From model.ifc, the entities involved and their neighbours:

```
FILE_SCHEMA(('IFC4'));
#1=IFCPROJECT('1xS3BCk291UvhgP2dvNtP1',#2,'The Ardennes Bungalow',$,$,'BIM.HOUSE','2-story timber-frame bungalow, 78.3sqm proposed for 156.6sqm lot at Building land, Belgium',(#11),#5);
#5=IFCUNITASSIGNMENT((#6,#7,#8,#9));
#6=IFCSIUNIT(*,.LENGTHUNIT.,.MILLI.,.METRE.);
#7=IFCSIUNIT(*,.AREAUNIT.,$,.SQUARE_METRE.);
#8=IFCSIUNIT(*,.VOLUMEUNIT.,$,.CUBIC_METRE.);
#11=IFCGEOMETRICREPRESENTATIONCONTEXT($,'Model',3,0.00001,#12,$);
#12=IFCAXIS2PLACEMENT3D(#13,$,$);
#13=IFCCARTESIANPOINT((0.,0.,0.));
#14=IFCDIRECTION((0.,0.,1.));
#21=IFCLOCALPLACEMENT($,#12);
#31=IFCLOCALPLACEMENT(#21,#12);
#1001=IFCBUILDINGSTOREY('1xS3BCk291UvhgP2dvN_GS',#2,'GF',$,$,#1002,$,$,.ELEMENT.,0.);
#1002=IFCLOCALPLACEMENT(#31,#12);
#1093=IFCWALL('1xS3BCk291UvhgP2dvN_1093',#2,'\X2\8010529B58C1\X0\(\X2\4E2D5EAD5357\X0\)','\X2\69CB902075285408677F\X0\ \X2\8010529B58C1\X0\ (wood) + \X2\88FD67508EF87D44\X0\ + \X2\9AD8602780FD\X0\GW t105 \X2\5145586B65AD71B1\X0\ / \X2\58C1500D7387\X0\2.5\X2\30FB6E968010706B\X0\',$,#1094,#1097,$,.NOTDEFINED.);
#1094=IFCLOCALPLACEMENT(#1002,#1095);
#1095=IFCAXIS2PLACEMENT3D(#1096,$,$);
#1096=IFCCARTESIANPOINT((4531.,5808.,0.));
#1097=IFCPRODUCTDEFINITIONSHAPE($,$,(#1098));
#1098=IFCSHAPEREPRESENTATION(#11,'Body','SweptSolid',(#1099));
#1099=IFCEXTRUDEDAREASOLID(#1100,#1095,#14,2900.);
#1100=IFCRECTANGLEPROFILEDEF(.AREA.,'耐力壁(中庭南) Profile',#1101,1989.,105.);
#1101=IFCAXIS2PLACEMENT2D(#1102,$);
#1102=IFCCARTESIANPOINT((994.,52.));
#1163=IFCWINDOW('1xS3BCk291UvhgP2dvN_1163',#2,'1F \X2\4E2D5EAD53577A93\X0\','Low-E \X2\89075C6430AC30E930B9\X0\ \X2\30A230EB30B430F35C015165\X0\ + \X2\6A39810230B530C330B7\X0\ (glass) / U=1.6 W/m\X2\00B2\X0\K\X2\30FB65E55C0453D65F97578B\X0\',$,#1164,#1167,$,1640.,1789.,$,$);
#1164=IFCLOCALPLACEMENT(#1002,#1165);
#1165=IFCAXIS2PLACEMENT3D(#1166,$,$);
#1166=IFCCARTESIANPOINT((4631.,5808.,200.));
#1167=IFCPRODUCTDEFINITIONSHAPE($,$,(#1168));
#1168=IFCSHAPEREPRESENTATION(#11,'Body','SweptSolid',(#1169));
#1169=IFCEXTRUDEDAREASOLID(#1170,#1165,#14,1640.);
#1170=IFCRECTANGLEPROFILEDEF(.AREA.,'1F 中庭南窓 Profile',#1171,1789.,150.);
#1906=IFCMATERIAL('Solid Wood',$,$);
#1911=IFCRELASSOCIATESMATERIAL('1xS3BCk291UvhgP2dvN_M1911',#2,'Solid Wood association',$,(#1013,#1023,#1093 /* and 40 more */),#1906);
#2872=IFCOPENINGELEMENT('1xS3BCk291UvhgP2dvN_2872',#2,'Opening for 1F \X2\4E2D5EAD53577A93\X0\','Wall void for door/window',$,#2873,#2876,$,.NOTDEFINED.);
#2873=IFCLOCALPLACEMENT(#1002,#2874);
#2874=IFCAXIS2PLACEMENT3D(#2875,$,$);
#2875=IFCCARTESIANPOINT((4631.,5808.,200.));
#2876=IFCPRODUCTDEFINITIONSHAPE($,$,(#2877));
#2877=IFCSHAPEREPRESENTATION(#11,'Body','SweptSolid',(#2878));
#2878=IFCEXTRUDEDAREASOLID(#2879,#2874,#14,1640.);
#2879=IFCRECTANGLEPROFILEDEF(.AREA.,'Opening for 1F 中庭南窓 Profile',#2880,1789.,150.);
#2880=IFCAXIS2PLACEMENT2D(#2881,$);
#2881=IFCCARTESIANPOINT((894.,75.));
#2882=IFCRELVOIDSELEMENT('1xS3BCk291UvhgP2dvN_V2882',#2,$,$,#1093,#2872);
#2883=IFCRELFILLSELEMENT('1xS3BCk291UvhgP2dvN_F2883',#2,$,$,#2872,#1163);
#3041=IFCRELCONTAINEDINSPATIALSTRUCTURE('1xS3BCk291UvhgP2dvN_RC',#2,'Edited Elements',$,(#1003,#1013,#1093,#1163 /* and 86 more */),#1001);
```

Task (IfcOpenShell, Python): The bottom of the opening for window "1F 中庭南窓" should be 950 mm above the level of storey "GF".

```python
import numpy as np
import ifcopenshell
import ifcopenshell.api.geometry
import ifcopenshell.geom
import ifcopenshell.util.element
import ifcopenshell.util.placement
import ifcopenshell.util.shape
import ifcopenshell.util.unit

model = ifcopenshell.open("model.ifc")
unit_scale = ifcopenshell.util.unit.calculate_unit_scale(model)

window = model.by_guid("1xS3BCk291UvhgP2dvN_1163")
opening = window.FillsVoids[0].RelatingOpeningElement
storey = ifcopenshell.util.element.get_container(window, ifc_class="IfcBuildingStorey")
level = ifcopenshell.util.placement.get_local_placement(storey.ObjectPlacement)[2, 3]

# The opening's origin need not be at the sill, so measure its lowest point.
shape = ifcopenshell.geom.create_shape(ifcopenshell.geom.settings(), opening)
bottom = ifcopenshell.util.shape.get_shape_bottom_elevation(shape, shape.geometry) / unit_scale
dz = level + 0.95 / unit_scale - bottom

shift = np.array([0.0, 0.0, dz])
# The window is not placed relative to its opening, so move both.
for product in (opening, window):
    matrix = ifcopenshell.util.placement.get_local_placement(product.ObjectPlacement)
    matrix[:3, 3] += shift
    ifcopenshell.api.geometry.edit_object_placement(model, product=product, matrix=matrix, is_si=False)

print(f"moved by {dz * unit_scale:+.3f} m")

model.write("model_updated.ifc")
```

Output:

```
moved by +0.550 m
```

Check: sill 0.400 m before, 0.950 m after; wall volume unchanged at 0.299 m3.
